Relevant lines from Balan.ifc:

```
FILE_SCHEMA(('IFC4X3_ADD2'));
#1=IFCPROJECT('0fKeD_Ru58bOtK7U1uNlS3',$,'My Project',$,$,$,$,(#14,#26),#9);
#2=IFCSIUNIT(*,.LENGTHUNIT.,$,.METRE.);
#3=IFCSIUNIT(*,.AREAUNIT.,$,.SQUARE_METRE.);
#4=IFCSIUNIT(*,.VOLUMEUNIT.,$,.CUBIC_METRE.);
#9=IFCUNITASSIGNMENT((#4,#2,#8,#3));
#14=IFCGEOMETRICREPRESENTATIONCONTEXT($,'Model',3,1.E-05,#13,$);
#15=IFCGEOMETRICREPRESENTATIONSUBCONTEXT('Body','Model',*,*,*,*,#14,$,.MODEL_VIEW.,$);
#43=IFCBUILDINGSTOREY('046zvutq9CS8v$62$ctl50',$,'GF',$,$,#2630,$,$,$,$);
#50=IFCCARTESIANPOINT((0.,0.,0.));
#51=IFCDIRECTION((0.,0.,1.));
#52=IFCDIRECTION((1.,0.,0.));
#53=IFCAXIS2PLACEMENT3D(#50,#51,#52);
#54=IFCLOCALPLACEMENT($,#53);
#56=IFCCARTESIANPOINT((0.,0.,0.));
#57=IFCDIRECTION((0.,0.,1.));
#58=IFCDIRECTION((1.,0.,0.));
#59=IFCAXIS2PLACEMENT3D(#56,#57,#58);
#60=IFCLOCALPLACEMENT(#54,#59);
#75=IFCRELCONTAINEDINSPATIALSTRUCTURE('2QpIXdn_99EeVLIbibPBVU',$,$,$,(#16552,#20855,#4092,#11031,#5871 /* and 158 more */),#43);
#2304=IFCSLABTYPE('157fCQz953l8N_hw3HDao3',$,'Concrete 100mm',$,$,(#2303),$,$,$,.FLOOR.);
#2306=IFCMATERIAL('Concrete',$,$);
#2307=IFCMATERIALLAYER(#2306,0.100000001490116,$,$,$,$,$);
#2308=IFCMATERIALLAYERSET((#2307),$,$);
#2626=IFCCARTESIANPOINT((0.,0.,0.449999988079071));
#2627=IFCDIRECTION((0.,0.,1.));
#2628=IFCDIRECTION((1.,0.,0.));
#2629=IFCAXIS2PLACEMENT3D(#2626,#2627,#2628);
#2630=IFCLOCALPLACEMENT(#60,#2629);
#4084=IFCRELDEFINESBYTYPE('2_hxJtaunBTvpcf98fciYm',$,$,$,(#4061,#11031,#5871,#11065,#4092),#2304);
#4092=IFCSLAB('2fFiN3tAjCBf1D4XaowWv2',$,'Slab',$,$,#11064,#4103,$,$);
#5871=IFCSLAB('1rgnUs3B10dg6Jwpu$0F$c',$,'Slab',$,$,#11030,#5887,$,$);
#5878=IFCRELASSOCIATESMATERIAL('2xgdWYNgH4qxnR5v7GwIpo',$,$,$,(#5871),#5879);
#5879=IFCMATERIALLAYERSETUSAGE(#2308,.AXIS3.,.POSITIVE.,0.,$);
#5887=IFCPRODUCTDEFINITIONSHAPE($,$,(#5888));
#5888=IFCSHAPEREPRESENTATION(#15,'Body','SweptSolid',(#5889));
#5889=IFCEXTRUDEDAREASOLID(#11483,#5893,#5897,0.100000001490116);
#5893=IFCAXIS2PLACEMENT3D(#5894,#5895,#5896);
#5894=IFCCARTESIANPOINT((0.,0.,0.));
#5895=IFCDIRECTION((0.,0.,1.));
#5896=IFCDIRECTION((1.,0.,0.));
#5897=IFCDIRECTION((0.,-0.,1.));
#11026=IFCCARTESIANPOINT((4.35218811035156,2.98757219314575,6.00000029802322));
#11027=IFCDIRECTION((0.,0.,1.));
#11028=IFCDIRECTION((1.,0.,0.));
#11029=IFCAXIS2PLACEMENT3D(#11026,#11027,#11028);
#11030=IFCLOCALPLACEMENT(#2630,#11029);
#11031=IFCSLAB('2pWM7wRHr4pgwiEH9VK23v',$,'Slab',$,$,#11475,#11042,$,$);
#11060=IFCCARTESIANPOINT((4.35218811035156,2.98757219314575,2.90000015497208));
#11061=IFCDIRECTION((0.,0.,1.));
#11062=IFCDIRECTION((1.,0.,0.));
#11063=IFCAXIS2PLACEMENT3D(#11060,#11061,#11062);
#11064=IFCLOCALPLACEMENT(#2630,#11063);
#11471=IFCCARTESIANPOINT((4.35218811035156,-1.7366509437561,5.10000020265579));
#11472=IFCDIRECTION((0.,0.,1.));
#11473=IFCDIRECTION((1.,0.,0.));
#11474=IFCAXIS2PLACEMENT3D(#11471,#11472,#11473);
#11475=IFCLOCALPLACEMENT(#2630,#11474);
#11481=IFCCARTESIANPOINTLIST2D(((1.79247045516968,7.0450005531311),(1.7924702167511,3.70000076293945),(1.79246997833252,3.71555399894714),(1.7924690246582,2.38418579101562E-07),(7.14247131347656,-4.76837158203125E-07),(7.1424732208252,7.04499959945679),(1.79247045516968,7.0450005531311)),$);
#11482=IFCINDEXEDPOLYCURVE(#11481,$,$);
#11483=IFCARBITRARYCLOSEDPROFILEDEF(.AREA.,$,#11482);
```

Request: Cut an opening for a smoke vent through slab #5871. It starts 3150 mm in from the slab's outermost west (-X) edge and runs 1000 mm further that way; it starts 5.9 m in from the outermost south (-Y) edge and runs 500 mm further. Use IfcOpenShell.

```python
import numpy as np
import ifcopenshell
import ifcopenshell.api.feature
import ifcopenshell.api.geometry
import ifcopenshell.api.root
import ifcopenshell.geom
import ifcopenshell.util.placement
import ifcopenshell.util.representation
import ifcopenshell.util.shape
import ifcopenshell.util.unit

model = ifcopenshell.open("Balan.ifc")
unit_scale = ifcopenshell.util.unit.calculate_unit_scale(model)
settings = ifcopenshell.geom.settings()


def volume(element):
    """Net volume in cubic metres, openings subtracted."""
    shape = ifcopenshell.geom.create_shape(settings, element)
    return ifcopenshell.util.shape.get_volume(shape.geometry)


slab = model.by_guid("1rgnUs3B10dg6Jwpu$0F$c")
before = volume(slab)

# Extent in the slab's own axes, in metres. The edges named are its -X and -Y sides.
slab_shape = ifcopenshell.geom.create_shape(settings, slab)
vertices = ifcopenshell.util.shape.get_vertices(slab_shape.geometry)
x_min, y_min, bottom = vertices.min(axis=0)
top = vertices[:, 2].max()

opening = ifcopenshell.api.root.create_entity(model, ifc_class="IfcOpeningElement", name="Smoke vent opening", predefined_type="OPENING")
context = ifcopenshell.util.representation.get_context(model, "Model", "Body", "MODEL_VIEW")
width, depth = 1, 0.5
outline = [(0.0, 0.0), (width, 0.0), (width, depth), (0.0, depth), (0.0, 0.0)]
# Overshoot both faces by 50 mm so the cut is clean.
shape = ifcopenshell.api.geometry.add_slab_representation(
    model, context=context, depth=top - bottom + 0.1, polyline=outline
)
ifcopenshell.api.geometry.assign_representation(model, product=opening, representation=shape)

matrix = ifcopenshell.util.placement.get_local_placement(slab.ObjectPlacement)
matrix[:, 3] = matrix @ np.append(np.array([x_min + 3.15, y_min + 5.9, bottom - 0.05]) / unit_scale, 1.0)
ifcopenshell.api.geometry.edit_object_placement(model, product=opening, matrix=matrix, is_si=False)
ifcopenshell.api.feature.add_feature(model, feature=opening, element=slab)

after = volume(slab)

print(f"slab volume {before:.3f} -> {after:.3f} m3")

model.write("Balan_v2.ifc")
```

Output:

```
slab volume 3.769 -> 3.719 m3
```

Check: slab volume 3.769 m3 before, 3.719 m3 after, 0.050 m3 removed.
